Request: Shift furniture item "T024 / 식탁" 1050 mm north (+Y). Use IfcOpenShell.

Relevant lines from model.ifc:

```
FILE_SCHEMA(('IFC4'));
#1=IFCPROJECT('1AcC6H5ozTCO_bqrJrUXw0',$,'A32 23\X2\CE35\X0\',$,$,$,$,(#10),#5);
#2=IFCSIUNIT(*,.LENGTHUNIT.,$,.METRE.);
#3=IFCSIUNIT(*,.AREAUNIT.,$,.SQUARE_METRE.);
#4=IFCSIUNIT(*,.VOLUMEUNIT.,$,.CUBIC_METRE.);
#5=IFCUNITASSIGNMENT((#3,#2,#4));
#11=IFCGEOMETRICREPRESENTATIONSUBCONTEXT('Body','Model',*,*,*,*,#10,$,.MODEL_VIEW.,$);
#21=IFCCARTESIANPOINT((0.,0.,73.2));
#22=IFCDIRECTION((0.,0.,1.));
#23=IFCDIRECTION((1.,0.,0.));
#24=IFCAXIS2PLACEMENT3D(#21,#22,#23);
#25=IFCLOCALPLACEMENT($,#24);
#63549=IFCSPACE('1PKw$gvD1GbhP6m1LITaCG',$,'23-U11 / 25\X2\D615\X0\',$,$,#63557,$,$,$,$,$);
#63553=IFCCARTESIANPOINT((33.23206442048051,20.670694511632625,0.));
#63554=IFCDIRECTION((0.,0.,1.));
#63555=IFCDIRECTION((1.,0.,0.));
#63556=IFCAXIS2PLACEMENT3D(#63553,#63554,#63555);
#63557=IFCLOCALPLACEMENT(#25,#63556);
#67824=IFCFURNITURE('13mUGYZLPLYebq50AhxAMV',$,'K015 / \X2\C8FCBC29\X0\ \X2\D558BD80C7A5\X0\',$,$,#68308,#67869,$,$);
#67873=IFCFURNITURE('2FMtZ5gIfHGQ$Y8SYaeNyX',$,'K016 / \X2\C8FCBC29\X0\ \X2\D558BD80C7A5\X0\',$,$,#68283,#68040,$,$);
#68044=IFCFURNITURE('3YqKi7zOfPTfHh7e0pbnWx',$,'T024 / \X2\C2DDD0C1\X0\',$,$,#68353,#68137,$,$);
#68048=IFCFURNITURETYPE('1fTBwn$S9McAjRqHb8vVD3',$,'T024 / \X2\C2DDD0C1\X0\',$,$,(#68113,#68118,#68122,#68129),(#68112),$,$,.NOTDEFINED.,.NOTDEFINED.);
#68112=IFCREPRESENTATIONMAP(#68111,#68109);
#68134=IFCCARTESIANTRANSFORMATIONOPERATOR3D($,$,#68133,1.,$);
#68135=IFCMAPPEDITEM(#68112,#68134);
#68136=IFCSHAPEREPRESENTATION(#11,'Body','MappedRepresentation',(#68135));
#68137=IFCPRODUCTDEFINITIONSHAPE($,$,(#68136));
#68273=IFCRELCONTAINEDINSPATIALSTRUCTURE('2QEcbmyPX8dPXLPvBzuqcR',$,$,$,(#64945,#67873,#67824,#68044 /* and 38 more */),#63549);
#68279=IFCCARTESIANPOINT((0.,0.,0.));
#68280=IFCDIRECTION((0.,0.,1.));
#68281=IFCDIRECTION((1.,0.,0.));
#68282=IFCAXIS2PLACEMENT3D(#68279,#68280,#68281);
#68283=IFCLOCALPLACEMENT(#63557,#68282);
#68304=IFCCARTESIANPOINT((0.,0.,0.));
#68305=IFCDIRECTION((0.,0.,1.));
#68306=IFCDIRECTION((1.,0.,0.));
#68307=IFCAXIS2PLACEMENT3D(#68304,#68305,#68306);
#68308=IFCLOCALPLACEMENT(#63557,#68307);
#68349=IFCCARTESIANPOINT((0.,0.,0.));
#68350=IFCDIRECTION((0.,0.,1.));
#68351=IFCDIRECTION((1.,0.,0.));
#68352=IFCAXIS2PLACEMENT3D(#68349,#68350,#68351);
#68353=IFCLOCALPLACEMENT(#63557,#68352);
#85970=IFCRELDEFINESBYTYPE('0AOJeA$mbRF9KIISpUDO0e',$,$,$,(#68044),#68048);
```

```python
import ifcopenshell
import ifcopenshell.api.geometry
import ifcopenshell.util.placement
import ifcopenshell.util.unit

model = ifcopenshell.open("model.ifc")
unit_scale = ifcopenshell.util.unit.calculate_unit_scale(model)

item = model.by_guid("3YqKi7zOfPTfHh7e0pbnWx")
matrix = ifcopenshell.util.placement.get_local_placement(item.ObjectPlacement)
matrix[1, 3] += 1.05 / unit_scale
ifcopenshell.api.geometry.edit_object_placement(model, product=item, matrix=matrix, is_si=False)

print(ifcopenshell.util.placement.get_local_placement(item.ObjectPlacement).round(3) + 0.0)

model.write("model_edited.ifc")
```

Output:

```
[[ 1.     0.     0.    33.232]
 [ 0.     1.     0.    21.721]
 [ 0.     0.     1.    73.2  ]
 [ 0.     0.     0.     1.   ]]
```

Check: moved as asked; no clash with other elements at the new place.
